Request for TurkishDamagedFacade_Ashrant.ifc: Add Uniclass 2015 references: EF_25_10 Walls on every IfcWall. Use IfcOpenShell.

First a look at what the model holds.

```python
import ifcopenshell

model = ifcopenshell.open("TurkishDamagedFacade_Ashrant.ifc")
print(model.schema)
print("classifications:", [c.Name for c in model.by_type("IfcClassification")])
for ifc_class in ("IfcDoor", "IfcRoof", "IfcStair", "IfcWall", "IfcWindow"):
    print(ifc_class, len(model.by_type(ifc_class)))
```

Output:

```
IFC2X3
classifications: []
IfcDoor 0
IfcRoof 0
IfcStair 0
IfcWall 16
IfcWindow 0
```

```python
import ifcopenshell
import ifcopenshell.api.classification

model = ifcopenshell.open("TurkishDamagedFacade_Ashrant.ifc")

# IFC2X3 requires Source and Edition and has no link from the project to the system.
system = model.create_entity("IfcClassification", Source="NBS", Edition="2015", Name="Uniclass 2015")

codes = {
    "IfcWall": ("EF_25_10", "Walls"),
}
for ifc_class, (code, name) in codes.items():
    products = model.by_type(ifc_class)
    ifcopenshell.api.classification.add_reference(
        model, products=products, classification=system, identification=code, name=name
    )
    print(code, len(products))

model.write("TurkishDamagedFacade_Ashrant_rev.ifc")
```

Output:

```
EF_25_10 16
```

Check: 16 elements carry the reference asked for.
